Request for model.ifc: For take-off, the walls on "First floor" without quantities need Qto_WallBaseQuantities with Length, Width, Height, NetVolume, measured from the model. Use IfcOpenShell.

First a look at what the model holds.

```python
import ifcopenshell
import ifcopenshell.util.element
import ifcopenshell.util.unit

model = ifcopenshell.open("model.ifc")
print(model.schema)
for unit_type in ("LENGTHUNIT", "AREAUNIT", "VOLUMEUNIT"):
    print(unit_type, ifcopenshell.util.unit.calculate_unit_scale(model, unit_type))
storey = next(s for s in model.by_type("IfcBuildingStorey") if s.Name == "First floor")
walls = [e for e in ifcopenshell.util.element.get_decomposition(storey) if e.is_a("IfcWall")]
for e in sorted(walls, key=lambda e: e.id()):
    print(e.id(), e.is_a(), e.Name, list(ifcopenshell.util.element.get_psets(e, qtos_only=True)), sep=" | ")
```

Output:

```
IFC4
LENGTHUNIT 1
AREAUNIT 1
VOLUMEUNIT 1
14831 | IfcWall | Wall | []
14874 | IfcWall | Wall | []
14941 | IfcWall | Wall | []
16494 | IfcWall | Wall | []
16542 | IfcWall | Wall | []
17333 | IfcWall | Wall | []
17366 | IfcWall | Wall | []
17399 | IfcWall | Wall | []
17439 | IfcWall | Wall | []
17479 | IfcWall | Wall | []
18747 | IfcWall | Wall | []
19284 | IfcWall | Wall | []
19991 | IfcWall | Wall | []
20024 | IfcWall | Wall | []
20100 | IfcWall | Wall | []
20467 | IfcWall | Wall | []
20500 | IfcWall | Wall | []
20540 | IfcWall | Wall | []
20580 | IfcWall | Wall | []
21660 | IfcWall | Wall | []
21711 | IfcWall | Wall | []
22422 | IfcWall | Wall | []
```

```python
import ifcopenshell
import ifcopenshell.api.pset
import ifcopenshell.geom
import ifcopenshell.util.element
import ifcopenshell.util.shape
import ifcopenshell.util.unit

model = ifcopenshell.open("model.ifc")
unit_scale = ifcopenshell.util.unit.calculate_unit_scale(model)
volume_scale = ifcopenshell.util.unit.calculate_unit_scale(model, "VOLUMEUNIT")
settings = ifcopenshell.geom.settings()

storey = next(s for s in model.by_type("IfcBuildingStorey") if s.Name == "First floor")
walls = [e for e in ifcopenshell.util.element.get_decomposition(storey) if e.is_a("IfcWall")]

for e in sorted(walls, key=lambda e: e.id()):
    if ifcopenshell.util.element.get_psets(e, qtos_only=True, should_inherit=False):
        continue
    # Geometry comes back in metres, in the element's own axes.
    shape = ifcopenshell.geom.create_shape(settings, e)
    values = {
        "Length": ifcopenshell.util.shape.get_x(shape.geometry) / unit_scale,
        "Width": ifcopenshell.util.shape.get_y(shape.geometry) / unit_scale,
        "Height": ifcopenshell.util.shape.get_z(shape.geometry) / unit_scale,
        "NetVolume": ifcopenshell.util.shape.get_volume(shape.geometry) / volume_scale,
    }
    qto = ifcopenshell.api.pset.add_qto(model, product=e, name="Qto_WallBaseQuantities")
    ifcopenshell.api.pset.edit_qto(model, qto=qto, properties=values)
    print(e.id(), {k: round(v, 3) for k, v in values.items()})

model.write("model_v2.ifc")
```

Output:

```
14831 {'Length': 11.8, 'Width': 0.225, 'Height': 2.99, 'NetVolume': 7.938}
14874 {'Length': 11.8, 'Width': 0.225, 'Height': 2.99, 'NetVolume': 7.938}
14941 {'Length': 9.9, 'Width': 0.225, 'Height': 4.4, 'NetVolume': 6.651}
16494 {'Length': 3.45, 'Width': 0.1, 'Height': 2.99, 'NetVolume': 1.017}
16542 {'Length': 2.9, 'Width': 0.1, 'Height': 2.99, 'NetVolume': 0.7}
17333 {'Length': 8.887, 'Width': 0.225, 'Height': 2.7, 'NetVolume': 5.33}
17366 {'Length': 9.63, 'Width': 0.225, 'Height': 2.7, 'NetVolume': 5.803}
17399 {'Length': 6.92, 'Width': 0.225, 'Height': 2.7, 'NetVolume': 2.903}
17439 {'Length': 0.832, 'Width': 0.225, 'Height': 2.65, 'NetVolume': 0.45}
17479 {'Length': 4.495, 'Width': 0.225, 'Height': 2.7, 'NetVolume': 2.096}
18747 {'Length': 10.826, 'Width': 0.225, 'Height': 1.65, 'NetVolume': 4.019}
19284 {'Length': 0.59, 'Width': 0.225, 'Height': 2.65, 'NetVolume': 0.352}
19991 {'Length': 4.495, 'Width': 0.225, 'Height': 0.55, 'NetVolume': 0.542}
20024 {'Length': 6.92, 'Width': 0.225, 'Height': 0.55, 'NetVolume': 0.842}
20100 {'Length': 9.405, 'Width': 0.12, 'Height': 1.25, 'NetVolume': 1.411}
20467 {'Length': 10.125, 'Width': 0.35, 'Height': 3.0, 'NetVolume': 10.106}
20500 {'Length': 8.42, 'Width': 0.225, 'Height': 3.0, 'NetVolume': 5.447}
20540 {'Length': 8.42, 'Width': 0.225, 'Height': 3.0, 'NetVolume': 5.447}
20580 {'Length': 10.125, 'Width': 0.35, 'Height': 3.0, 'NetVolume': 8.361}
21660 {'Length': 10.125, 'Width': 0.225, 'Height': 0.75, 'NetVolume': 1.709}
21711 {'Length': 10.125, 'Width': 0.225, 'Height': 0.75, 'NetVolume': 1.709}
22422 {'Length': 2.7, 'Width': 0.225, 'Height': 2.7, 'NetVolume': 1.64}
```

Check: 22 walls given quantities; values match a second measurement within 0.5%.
